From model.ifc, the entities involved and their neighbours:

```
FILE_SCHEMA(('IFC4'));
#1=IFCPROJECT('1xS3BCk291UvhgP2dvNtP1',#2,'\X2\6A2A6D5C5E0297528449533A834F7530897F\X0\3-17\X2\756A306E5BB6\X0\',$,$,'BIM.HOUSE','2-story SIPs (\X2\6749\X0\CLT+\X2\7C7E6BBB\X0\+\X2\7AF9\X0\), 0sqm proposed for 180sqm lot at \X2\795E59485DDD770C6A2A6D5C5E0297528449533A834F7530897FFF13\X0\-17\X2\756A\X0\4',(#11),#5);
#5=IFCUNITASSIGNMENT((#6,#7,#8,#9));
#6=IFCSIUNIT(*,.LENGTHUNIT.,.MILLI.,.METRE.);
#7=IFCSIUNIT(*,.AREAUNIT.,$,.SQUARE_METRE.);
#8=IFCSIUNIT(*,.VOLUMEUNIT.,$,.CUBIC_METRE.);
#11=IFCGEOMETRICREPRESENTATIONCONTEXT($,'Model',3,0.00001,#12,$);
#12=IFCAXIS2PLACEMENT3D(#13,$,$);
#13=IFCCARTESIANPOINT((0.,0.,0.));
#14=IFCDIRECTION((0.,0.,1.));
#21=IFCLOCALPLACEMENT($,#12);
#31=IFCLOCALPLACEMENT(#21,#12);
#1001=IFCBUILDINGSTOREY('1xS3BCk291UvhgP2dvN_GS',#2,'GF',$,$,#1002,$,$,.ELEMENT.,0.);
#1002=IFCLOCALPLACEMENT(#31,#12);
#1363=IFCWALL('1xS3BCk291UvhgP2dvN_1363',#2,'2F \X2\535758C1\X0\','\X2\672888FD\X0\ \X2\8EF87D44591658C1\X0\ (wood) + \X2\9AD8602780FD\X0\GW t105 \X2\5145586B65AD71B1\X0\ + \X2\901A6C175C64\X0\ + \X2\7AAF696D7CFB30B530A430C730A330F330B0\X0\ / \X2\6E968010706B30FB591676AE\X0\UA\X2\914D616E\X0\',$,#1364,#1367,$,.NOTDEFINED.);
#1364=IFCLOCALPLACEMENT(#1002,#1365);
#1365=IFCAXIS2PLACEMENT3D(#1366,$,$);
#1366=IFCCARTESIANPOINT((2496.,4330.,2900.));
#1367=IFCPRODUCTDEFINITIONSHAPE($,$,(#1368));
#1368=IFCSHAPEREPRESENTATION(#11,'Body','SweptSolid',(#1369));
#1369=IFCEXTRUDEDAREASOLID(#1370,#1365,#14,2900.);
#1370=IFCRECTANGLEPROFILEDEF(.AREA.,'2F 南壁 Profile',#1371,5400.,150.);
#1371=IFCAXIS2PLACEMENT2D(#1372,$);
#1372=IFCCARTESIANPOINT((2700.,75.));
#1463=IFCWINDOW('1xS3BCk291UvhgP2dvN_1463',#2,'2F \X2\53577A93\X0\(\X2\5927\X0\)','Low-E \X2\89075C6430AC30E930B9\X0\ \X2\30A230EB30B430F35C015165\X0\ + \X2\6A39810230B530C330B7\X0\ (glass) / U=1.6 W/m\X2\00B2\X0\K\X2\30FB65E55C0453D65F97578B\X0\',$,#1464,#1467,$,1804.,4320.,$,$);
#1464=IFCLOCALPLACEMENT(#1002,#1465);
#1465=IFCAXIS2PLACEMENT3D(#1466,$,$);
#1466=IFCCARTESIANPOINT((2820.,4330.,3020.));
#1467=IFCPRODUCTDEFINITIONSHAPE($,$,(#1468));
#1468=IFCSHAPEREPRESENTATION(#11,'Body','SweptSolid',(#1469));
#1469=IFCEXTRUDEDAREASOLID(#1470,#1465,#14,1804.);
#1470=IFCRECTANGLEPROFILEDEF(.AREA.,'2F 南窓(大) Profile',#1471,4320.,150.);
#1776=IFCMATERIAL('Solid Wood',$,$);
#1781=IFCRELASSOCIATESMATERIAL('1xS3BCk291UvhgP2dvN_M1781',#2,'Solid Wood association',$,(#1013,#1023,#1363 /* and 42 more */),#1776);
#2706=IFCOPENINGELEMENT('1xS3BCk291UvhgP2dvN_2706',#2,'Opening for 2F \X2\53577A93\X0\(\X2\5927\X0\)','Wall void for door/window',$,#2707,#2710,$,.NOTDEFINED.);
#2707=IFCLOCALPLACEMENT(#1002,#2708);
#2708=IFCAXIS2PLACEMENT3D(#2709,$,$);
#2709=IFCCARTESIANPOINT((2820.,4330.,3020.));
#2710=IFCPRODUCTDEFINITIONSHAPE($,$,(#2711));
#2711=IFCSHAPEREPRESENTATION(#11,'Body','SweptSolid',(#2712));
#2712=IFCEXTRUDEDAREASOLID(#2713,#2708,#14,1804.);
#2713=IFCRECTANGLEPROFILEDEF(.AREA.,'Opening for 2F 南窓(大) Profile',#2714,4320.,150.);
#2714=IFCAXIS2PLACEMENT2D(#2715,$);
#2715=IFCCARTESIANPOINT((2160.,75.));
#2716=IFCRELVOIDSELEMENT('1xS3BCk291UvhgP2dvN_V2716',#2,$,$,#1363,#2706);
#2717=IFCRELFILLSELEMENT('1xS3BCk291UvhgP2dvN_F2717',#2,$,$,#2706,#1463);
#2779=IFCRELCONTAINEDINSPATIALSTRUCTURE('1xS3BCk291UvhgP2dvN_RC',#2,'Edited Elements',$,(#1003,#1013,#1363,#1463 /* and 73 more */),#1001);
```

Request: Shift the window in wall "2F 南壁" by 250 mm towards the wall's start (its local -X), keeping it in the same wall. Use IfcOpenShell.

```python
import ifcopenshell
import ifcopenshell.api.geometry
import ifcopenshell.util.placement
import ifcopenshell.util.unit

model = ifcopenshell.open("model.ifc")
unit_scale = ifcopenshell.util.unit.calculate_unit_scale(model)

window = model.by_guid("1xS3BCk291UvhgP2dvN_1463")
opening = window.FillsVoids[0].RelatingOpeningElement
wall = opening.VoidsElements[0].RelatingBuildingElement

wall_matrix = ifcopenshell.util.placement.get_local_placement(wall.ObjectPlacement)
shift = wall_matrix[:3, 0] * -0.25 / unit_scale
before = ifcopenshell.util.placement.get_local_placement(window.ObjectPlacement)[:3, 3].copy()

# The window is not placed relative to its opening, so move both.
for product in (opening, window):
    matrix = ifcopenshell.util.placement.get_local_placement(product.ObjectPlacement)
    matrix[:3, 3] += shift
    ifcopenshell.api.geometry.edit_object_placement(model, product=product, matrix=matrix, is_si=False)

after = ifcopenshell.util.placement.get_local_placement(window.ObjectPlacement)[:3, 3]
print("window moved by", (after - before).round(3) + 0.0)

model.write("model_rev.ifc")
```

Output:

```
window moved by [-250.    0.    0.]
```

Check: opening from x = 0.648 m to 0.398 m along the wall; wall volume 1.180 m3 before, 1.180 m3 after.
